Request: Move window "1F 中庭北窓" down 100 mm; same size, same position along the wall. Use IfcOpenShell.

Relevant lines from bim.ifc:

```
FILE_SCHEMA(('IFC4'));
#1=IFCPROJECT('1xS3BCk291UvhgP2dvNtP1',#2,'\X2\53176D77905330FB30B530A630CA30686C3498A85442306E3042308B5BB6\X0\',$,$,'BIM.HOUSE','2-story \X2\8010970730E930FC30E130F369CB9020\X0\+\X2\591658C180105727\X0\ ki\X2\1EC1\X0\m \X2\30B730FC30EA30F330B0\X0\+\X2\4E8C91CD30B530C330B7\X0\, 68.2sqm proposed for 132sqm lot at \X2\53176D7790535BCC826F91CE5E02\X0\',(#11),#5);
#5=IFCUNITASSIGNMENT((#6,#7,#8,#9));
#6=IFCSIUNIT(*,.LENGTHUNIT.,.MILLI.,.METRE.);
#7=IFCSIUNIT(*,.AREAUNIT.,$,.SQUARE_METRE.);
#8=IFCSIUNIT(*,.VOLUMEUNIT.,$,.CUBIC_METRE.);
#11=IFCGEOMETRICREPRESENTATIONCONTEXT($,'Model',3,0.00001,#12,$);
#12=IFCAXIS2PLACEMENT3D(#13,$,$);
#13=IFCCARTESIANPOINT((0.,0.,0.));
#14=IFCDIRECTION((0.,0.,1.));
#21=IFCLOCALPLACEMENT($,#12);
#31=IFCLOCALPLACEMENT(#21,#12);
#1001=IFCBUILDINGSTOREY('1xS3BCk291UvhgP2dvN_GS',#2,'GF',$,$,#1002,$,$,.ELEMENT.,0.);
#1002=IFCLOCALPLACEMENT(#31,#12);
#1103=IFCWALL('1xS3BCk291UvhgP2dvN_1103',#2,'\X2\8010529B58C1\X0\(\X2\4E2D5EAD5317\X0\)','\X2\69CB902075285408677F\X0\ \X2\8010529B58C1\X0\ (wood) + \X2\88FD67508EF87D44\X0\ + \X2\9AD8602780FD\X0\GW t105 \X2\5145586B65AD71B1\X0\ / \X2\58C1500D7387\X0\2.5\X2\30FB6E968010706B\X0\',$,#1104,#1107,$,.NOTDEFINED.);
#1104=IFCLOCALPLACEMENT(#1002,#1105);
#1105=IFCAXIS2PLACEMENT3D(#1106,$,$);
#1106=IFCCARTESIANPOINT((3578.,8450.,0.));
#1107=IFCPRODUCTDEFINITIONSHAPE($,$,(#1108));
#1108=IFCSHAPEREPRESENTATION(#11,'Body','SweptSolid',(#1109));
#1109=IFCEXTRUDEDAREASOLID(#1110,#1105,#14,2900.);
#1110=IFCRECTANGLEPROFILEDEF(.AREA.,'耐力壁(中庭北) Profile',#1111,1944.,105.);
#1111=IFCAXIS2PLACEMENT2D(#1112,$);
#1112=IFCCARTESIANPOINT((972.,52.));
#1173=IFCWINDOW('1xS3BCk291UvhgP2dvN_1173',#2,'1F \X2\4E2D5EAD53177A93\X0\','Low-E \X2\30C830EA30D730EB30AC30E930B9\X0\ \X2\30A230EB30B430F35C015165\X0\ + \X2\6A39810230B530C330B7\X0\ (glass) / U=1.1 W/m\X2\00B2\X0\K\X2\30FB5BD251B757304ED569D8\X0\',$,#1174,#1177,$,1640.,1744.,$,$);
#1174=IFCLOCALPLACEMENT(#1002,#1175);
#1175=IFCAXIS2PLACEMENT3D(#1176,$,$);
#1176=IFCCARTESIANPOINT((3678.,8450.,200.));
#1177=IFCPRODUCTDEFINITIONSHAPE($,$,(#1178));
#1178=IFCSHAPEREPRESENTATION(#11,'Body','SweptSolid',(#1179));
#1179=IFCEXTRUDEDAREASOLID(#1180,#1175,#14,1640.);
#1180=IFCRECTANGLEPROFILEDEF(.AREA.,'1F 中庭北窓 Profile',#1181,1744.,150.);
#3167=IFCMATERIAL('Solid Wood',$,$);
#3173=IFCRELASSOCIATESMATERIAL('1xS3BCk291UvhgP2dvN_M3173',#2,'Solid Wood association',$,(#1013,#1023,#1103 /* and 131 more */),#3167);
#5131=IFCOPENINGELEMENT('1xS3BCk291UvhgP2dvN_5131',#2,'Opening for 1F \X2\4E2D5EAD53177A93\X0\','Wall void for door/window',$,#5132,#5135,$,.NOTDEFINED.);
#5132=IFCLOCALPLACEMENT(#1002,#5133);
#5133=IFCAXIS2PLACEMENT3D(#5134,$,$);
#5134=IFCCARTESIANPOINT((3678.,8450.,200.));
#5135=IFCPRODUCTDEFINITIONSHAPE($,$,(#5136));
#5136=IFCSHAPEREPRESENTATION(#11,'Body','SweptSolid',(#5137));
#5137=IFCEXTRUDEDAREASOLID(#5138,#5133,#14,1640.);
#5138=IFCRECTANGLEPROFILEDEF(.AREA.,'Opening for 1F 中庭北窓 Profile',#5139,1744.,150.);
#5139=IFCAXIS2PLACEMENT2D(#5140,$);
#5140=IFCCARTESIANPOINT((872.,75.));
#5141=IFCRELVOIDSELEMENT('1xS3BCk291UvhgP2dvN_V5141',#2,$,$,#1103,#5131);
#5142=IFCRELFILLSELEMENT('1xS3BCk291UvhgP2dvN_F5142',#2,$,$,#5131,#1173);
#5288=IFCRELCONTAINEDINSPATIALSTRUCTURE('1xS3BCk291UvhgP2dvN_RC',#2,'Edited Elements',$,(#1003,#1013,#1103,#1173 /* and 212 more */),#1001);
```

```python
import numpy as np
import ifcopenshell
import ifcopenshell.api.geometry
import ifcopenshell.util.placement
import ifcopenshell.util.unit

model = ifcopenshell.open("bim.ifc")
unit_scale = ifcopenshell.util.unit.calculate_unit_scale(model)

window = model.by_id(1173)
opening = window.FillsVoids[0].RelatingOpeningElement
dz = -0.1 / unit_scale

shift = np.array([0.0, 0.0, dz])
# The window is not placed relative to its opening, so move both.
for product in (opening, window):
    matrix = ifcopenshell.util.placement.get_local_placement(product.ObjectPlacement)
    matrix[:3, 3] += shift
    ifcopenshell.api.geometry.edit_object_placement(model, product=product, matrix=matrix, is_si=False)

print(f"moved by {dz * unit_scale:+.3f} m")

model.write("bim_updated.ifc")
```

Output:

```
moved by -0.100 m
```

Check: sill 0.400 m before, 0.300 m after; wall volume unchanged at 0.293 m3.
